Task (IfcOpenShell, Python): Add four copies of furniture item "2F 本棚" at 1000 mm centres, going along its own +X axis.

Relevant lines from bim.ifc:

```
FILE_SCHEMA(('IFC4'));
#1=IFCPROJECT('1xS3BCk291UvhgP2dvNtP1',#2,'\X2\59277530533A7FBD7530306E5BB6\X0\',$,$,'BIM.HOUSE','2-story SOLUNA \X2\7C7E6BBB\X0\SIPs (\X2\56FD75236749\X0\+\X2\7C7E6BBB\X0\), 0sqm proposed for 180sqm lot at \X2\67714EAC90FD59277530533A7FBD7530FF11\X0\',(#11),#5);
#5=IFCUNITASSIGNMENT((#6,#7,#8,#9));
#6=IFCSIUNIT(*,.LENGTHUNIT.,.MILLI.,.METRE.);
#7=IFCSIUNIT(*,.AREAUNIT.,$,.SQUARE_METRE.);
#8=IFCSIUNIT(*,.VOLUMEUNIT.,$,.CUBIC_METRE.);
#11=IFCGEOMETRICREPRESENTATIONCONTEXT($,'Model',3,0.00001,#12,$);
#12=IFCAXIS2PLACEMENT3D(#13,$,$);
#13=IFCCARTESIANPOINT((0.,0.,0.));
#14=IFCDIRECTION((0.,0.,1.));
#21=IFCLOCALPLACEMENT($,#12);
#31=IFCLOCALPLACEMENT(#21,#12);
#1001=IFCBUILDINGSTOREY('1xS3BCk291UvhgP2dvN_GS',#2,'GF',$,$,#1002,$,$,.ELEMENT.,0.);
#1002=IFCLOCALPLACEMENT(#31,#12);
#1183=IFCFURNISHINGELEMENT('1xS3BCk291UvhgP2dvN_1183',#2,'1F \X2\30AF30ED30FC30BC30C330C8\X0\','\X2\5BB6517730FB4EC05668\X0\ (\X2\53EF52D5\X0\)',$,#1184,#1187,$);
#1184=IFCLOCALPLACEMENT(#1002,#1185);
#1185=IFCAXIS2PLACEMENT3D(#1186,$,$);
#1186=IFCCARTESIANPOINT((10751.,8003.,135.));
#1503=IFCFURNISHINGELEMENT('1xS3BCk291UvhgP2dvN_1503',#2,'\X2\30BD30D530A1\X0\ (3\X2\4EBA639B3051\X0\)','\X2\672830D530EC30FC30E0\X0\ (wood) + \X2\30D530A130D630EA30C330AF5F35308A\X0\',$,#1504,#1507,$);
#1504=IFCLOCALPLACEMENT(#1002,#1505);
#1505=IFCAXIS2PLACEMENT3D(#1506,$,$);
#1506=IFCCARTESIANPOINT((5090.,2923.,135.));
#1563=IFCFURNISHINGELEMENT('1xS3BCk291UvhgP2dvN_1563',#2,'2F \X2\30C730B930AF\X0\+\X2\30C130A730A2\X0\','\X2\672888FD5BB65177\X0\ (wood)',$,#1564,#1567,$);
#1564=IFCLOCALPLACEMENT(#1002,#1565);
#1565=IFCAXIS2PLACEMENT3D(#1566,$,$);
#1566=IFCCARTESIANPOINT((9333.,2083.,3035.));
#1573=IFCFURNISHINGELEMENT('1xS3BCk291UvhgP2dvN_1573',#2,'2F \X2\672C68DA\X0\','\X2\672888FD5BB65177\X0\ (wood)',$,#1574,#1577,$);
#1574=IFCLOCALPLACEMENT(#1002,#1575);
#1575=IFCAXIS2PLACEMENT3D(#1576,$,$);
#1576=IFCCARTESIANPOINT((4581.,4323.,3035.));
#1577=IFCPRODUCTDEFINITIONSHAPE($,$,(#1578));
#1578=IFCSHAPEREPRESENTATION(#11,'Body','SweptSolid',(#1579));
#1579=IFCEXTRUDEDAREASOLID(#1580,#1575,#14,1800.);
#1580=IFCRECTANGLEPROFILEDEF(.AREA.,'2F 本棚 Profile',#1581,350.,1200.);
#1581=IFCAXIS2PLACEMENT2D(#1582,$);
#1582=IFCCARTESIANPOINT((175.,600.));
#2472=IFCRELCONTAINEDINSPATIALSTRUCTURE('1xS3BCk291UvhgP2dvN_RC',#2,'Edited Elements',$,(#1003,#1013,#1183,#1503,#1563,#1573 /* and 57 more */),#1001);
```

```python
import ifcopenshell
import ifcopenshell.api.geometry
import ifcopenshell.api.root
import ifcopenshell.util.element
import ifcopenshell.util.placement

model = ifcopenshell.open("bim.ifc")


def reuse_history(source, copy):
    """copy_class also copies each property set's owner history, people and application; keep the originals."""
    for rel in copy.IsDefinedBy:
        if rel.is_a("IfcRelDefinesByProperties") and (history := rel.RelatingPropertyDefinition.OwnerHistory):
            rel.RelatingPropertyDefinition.OwnerHistory = source.OwnerHistory
            ifcopenshell.util.element.remove_deep2(model, history)


source = model.by_guid("1xS3BCk291UvhgP2dvN_1573")
base = ifcopenshell.util.placement.get_local_placement(source.ObjectPlacement)
step = base[:3, 0] * 1000.0

for i in range(1, 5):
    copy = ifcopenshell.api.root.copy_class(model, product=source)
    copy.Representation = ifcopenshell.util.element.copy_deep(
        model, source.Representation, exclude=["IfcGeometricRepresentationContext", "IfcRepresentationMap"]
    )
    reuse_history(source, copy)
    matrix = base.copy()
    matrix[:3, 3] += i * step
    print("added at", matrix[:3, 3].round(3) + 0.0)
    ifcopenshell.api.geometry.edit_object_placement(model, product=copy, matrix=matrix, is_si=False)

model.write("bim_rev.ifc")
```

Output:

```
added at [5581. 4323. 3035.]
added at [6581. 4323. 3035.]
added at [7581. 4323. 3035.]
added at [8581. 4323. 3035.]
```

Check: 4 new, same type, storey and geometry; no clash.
